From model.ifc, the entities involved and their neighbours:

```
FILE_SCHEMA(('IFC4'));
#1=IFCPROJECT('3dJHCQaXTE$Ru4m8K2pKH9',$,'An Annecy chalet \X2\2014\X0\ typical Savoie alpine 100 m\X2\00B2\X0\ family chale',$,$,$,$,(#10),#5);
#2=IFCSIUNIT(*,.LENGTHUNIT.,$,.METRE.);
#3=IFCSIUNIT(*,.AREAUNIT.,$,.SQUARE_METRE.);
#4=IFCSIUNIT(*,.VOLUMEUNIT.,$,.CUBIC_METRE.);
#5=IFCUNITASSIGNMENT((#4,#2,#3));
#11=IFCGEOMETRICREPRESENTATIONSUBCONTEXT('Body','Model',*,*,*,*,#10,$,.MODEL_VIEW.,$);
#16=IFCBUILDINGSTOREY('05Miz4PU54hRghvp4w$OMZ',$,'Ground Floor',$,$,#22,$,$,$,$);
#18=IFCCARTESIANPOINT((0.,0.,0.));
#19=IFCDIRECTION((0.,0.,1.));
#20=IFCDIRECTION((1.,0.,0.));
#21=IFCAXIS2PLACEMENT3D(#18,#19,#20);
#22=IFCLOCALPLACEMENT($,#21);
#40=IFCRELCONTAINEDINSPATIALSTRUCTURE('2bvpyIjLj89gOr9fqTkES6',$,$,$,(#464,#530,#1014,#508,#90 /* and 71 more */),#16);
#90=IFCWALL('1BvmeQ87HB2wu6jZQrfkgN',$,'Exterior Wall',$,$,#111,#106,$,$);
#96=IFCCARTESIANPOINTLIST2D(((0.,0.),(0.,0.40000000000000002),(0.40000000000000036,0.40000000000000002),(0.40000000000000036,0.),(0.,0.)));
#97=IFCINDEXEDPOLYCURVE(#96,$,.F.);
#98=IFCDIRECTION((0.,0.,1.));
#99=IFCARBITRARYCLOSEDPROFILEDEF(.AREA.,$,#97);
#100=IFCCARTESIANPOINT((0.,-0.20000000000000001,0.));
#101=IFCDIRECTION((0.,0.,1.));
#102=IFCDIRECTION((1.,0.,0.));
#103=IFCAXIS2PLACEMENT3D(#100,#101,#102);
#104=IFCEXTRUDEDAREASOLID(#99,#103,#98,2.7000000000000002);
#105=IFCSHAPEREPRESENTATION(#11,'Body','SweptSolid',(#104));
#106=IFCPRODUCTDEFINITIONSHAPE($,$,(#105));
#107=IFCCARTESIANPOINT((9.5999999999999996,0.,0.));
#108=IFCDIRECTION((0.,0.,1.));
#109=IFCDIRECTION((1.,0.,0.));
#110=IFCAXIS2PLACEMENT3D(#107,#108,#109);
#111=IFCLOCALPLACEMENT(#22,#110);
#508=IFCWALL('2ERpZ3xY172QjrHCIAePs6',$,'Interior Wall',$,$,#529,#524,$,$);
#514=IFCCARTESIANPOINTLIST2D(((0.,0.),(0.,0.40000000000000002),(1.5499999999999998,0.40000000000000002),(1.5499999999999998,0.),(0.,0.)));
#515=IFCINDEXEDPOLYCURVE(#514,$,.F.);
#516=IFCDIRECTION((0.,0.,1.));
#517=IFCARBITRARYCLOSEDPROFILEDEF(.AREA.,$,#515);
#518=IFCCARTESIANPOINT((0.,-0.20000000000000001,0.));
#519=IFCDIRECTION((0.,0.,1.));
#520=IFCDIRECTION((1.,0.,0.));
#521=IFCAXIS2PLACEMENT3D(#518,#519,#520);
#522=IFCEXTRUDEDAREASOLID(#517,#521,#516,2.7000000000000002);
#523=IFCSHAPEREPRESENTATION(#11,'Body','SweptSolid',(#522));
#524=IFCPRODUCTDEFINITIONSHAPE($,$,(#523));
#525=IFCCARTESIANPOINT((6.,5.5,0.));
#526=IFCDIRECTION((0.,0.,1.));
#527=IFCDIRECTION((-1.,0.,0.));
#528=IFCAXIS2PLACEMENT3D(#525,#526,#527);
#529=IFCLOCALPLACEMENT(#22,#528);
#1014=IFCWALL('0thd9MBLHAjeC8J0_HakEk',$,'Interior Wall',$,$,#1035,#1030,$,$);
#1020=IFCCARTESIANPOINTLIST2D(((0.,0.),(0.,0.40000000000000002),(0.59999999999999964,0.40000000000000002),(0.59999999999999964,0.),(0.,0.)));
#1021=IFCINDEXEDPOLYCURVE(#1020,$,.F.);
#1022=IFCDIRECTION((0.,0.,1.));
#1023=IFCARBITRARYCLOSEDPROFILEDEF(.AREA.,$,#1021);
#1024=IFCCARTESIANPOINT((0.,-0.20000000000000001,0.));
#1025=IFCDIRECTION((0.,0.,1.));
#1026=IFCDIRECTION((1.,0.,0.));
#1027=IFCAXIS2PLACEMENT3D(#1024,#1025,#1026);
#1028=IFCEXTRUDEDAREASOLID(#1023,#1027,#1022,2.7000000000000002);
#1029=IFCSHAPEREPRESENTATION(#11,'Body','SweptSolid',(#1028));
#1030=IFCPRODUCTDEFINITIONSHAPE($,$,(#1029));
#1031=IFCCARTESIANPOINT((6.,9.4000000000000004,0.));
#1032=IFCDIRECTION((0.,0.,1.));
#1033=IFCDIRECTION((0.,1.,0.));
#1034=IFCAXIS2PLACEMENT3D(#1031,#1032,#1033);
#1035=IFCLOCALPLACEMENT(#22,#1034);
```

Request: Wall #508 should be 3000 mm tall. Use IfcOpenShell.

```python
import ifcopenshell
import ifcopenshell.geom
import ifcopenshell.util.representation
import ifcopenshell.util.shape
import ifcopenshell.util.unit

model = ifcopenshell.open("model.ifc")
unit_scale = ifcopenshell.util.unit.calculate_unit_scale(model)
settings = ifcopenshell.geom.settings()


def volume(element):
    """Net volume in cubic metres, openings subtracted."""
    shape = ifcopenshell.geom.create_shape(settings, element)
    return ifcopenshell.util.shape.get_volume(shape.geometry)


wall = model.by_guid("2ERpZ3xY172QjrHCIAePs6")
before = volume(wall)

body = ifcopenshell.util.representation.get_representation(wall, "Model", "Body")
solid = body.Items[0]
old_height = solid.Depth
solid.Depth = 3 / unit_scale
after = volume(wall)

print(f"height {old_height:g} -> {solid.Depth:g}, volume {before:.3f} -> {after:.3f} m3")

model.write("model-out.ifc")
```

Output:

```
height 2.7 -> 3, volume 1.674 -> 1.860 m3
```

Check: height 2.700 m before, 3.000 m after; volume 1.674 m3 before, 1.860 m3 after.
